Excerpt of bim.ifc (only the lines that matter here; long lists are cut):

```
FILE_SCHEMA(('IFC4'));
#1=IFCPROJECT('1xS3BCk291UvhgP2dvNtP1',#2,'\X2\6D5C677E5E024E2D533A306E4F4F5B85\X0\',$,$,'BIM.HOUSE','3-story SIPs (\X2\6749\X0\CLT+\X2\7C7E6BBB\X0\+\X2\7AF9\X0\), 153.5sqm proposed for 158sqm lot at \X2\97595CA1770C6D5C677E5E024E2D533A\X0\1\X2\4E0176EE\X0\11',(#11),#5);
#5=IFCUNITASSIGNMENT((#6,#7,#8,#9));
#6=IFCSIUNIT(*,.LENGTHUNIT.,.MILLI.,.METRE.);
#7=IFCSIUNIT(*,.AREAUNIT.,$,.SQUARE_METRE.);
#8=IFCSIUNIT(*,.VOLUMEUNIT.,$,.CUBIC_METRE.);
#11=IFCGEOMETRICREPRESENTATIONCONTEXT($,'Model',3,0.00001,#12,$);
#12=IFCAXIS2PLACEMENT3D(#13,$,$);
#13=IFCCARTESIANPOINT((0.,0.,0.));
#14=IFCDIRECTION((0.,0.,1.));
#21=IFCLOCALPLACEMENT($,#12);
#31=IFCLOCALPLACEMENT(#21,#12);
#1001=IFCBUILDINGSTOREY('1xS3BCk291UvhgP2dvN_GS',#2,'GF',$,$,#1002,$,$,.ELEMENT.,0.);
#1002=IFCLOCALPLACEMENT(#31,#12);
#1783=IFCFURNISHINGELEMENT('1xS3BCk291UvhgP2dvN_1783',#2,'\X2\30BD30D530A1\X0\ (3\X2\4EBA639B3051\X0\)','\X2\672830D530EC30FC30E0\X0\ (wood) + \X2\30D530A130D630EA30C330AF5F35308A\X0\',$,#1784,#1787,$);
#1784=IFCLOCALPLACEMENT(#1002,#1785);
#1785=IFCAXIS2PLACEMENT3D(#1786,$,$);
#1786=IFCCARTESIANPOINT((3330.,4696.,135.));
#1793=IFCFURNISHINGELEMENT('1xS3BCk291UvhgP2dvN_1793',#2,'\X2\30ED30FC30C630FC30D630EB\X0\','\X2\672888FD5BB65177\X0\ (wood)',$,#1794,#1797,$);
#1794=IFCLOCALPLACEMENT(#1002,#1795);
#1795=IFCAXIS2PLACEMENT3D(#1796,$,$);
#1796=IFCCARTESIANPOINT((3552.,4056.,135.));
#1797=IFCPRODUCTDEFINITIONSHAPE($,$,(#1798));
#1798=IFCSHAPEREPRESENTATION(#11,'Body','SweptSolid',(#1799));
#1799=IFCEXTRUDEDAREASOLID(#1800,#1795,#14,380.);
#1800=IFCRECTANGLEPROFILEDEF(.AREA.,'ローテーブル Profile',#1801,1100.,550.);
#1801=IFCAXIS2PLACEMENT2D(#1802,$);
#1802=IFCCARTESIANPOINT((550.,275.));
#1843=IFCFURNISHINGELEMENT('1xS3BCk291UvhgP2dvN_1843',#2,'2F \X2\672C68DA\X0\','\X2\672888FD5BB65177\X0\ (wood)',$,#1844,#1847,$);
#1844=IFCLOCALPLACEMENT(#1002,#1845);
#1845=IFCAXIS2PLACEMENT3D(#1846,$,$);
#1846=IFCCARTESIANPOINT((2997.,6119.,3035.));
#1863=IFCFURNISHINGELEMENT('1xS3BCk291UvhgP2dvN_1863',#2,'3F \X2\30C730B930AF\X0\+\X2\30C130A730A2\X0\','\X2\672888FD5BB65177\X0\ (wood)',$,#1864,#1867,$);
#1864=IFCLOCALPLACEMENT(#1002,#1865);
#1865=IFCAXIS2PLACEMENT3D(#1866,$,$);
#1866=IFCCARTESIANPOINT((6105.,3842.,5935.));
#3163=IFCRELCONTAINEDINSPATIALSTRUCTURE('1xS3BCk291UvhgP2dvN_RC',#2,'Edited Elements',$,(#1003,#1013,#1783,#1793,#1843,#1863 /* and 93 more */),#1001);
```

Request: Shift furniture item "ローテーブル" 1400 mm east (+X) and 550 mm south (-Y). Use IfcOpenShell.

```python
import ifcopenshell
import ifcopenshell.api.geometry
import ifcopenshell.util.placement
import ifcopenshell.util.unit

model = ifcopenshell.open("bim.ifc")
unit_scale = ifcopenshell.util.unit.calculate_unit_scale(model)

item = model.by_guid("1xS3BCk291UvhgP2dvN_1793")
matrix = ifcopenshell.util.placement.get_local_placement(item.ObjectPlacement)
matrix[0, 3] += 1.4 / unit_scale
matrix[1, 3] -= 0.55 / unit_scale
ifcopenshell.api.geometry.edit_object_placement(model, product=item, matrix=matrix, is_si=False)

print(ifcopenshell.util.placement.get_local_placement(item.ObjectPlacement).round(3) + 0.0)

model.write("bim_updated.ifc")
```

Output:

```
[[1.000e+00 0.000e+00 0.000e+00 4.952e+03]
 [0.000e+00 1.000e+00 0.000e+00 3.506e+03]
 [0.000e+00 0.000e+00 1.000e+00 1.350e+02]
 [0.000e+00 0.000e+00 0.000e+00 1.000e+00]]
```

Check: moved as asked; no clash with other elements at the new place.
